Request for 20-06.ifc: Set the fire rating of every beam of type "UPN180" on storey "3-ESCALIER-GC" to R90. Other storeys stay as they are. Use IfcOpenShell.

First a look at what the model holds.

```python
import ifcopenshell
import ifcopenshell.util.element

model = ifcopenshell.open("20-06.ifc")
print(model.schema)
storey = next(s for s in model.by_type("IfcBuildingStorey") if s.Name == "3-ESCALIER-GC")
beams = [e for e in ifcopenshell.util.element.get_decomposition(storey) if e.is_a("IfcBeam")]
seen = {}
for e in beams:
    element_type = ifcopenshell.util.element.get_type(e)
    key = (element_type.Name if element_type != e and element_type else None, ifcopenshell.util.element.get_pset(e, "Pset_BeamCommon", "FireRating"))
    seen[key] = seen.get(key, 0) + 1
for (name, value), count in sorted(seen.items(), key=str):
    print(count, "x", name, "|", value)
```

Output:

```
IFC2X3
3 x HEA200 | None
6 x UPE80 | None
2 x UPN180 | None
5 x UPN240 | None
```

```python
import ifcopenshell
import ifcopenshell.api.pset
import ifcopenshell.util.element

model = ifcopenshell.open("20-06.ifc")

storey = next(s for s in model.by_type("IfcBuildingStorey") if s.Name == "3-ESCALIER-GC")
beams = [e for e in ifcopenshell.util.element.get_decomposition(storey) if e.is_a("IfcBeam")]

count = 0
for e in beams:
    element_type = ifcopenshell.util.element.get_type(e)
    if element_type in (None, e) or element_type.Name != "UPN180":
        continue
    # add_pset returns the element's existing set when there is one.
    pset = ifcopenshell.api.pset.add_pset(model, product=e, name="Pset_BeamCommon")
    ifcopenshell.api.pset.edit_pset(model, pset=pset, properties={"FireRating": "R90"})
    count += 1

print(count, "beams updated")

model.write("20-06_updated.ifc")
```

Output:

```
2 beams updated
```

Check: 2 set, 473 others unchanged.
